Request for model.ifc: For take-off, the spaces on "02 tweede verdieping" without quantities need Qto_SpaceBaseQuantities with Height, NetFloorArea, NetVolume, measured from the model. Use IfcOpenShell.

First a look at what the model holds.

```python
import ifcopenshell
import ifcopenshell.util.element
import ifcopenshell.util.unit

model = ifcopenshell.open("model.ifc")
print(model.schema)
for unit_type in ("LENGTHUNIT", "AREAUNIT", "VOLUMEUNIT"):
    print(unit_type, ifcopenshell.util.unit.calculate_unit_scale(model, unit_type))
storey = next(s for s in model.by_type("IfcBuildingStorey") if s.Name == "02 tweede verdieping")
spaces = [e for e in ifcopenshell.util.element.get_decomposition(storey) if e.is_a("IfcSpace")]
for e in sorted(spaces, key=lambda e: e.id()):
    print(e.id(), e.is_a(), e.Name, list(ifcopenshell.util.element.get_psets(e, qtos_only=True)), sep=" | ")
```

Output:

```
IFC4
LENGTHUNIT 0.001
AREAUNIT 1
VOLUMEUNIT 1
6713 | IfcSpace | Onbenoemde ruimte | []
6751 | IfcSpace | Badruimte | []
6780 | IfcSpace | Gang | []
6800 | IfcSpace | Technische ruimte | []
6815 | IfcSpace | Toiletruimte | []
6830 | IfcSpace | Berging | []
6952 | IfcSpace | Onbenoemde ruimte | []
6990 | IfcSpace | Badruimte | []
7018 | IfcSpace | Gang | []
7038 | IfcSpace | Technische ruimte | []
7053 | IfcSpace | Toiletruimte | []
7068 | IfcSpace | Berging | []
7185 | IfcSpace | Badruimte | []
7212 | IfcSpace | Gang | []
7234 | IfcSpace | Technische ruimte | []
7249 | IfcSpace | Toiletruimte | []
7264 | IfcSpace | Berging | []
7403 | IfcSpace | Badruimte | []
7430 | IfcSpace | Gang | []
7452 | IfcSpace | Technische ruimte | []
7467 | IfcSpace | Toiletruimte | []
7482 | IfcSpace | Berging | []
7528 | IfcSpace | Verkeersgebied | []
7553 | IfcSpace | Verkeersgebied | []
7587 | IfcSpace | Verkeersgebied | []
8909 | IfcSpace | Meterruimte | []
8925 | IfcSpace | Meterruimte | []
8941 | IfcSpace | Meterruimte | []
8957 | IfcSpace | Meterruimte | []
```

```python
import ifcopenshell
import ifcopenshell.api.pset
import ifcopenshell.geom
import ifcopenshell.util.element
import ifcopenshell.util.shape
import ifcopenshell.util.unit

model = ifcopenshell.open("model.ifc")
unit_scale = ifcopenshell.util.unit.calculate_unit_scale(model)
area_scale = ifcopenshell.util.unit.calculate_unit_scale(model, "AREAUNIT")
volume_scale = ifcopenshell.util.unit.calculate_unit_scale(model, "VOLUMEUNIT")
settings = ifcopenshell.geom.settings()

storey = next(s for s in model.by_type("IfcBuildingStorey") if s.Name == "02 tweede verdieping")
spaces = [e for e in ifcopenshell.util.element.get_decomposition(storey) if e.is_a("IfcSpace")]

for e in sorted(spaces, key=lambda e: e.id()):
    if ifcopenshell.util.element.get_psets(e, qtos_only=True, should_inherit=False):
        continue
    # Geometry comes back in metres, in the element's own axes.
    shape = ifcopenshell.geom.create_shape(settings, e)
    values = {
        "Height": ifcopenshell.util.shape.get_z(shape.geometry) / unit_scale,
        "NetFloorArea": ifcopenshell.util.shape.get_footprint_area(shape.geometry) / area_scale,
        "NetVolume": ifcopenshell.util.shape.get_volume(shape.geometry) / volume_scale,
    }
    qto = ifcopenshell.api.pset.add_qto(model, product=e, name="Qto_SpaceBaseQuantities")
    ifcopenshell.api.pset.edit_qto(model, qto=qto, properties=values)
    print(e.id(), {k: round(v, 3) for k, v in values.items()})

model.write("model_v2.ifc")
```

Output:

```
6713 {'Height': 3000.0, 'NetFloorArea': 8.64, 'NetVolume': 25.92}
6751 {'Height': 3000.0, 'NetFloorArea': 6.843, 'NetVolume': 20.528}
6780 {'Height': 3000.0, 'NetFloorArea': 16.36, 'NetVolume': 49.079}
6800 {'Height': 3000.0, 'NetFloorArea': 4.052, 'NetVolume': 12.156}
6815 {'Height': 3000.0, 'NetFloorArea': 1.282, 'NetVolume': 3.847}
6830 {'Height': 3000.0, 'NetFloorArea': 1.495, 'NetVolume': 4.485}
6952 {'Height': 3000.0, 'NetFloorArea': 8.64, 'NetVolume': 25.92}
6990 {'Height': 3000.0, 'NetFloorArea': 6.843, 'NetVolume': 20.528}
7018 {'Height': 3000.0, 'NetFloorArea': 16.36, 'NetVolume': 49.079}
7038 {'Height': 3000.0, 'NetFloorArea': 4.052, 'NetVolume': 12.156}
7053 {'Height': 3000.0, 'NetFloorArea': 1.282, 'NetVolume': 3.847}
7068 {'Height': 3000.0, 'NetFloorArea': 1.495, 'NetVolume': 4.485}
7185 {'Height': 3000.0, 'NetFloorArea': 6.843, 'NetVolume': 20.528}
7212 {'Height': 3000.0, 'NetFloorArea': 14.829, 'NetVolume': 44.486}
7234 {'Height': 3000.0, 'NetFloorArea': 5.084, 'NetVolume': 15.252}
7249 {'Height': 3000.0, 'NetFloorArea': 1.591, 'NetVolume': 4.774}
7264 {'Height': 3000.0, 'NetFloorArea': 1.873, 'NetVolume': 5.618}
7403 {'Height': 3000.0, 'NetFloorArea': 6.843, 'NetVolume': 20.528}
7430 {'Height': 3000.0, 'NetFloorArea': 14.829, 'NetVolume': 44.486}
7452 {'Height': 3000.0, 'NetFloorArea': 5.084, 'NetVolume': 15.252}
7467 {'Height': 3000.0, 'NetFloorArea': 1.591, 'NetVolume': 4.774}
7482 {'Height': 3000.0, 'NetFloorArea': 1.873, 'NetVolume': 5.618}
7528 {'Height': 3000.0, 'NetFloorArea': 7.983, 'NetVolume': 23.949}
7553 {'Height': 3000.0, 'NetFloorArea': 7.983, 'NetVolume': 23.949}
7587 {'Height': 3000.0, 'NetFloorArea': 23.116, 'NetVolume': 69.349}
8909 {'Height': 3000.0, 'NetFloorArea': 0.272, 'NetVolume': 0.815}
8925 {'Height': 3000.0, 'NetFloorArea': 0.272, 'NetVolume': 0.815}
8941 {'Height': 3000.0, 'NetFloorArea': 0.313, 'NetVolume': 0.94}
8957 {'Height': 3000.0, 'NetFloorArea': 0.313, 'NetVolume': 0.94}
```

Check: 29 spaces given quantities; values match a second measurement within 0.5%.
